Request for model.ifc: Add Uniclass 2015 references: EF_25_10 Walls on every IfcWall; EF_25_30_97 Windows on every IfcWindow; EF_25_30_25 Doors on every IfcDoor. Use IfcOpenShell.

First a look at what the model holds.

```python
import ifcopenshell

model = ifcopenshell.open("model.ifc")
print(model.schema)
print("classifications:", [c.Name for c in model.by_type("IfcClassification")])
for ifc_class in ("IfcDoor", "IfcRoof", "IfcStair", "IfcWall", "IfcWindow"):
    print(ifc_class, len(model.by_type(ifc_class)))
```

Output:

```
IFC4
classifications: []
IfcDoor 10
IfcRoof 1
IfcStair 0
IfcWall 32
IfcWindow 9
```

```python
import ifcopenshell
import ifcopenshell.api.classification

model = ifcopenshell.open("model.ifc")

system = ifcopenshell.api.classification.add_classification(model, classification="Uniclass 2015")

codes = {
    "IfcWall": ("EF_25_10", "Walls"),
    "IfcWindow": ("EF_25_30_97", "Windows"),
    "IfcDoor": ("EF_25_30_25", "Doors"),
}
for ifc_class, (code, name) in codes.items():
    products = model.by_type(ifc_class)
    ifcopenshell.api.classification.add_reference(
        model, products=products, classification=system, identification=code, name=name
    )
    print(code, len(products))

model.write("model_v2.ifc")
```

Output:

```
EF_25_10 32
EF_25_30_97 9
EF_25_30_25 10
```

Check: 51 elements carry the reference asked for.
